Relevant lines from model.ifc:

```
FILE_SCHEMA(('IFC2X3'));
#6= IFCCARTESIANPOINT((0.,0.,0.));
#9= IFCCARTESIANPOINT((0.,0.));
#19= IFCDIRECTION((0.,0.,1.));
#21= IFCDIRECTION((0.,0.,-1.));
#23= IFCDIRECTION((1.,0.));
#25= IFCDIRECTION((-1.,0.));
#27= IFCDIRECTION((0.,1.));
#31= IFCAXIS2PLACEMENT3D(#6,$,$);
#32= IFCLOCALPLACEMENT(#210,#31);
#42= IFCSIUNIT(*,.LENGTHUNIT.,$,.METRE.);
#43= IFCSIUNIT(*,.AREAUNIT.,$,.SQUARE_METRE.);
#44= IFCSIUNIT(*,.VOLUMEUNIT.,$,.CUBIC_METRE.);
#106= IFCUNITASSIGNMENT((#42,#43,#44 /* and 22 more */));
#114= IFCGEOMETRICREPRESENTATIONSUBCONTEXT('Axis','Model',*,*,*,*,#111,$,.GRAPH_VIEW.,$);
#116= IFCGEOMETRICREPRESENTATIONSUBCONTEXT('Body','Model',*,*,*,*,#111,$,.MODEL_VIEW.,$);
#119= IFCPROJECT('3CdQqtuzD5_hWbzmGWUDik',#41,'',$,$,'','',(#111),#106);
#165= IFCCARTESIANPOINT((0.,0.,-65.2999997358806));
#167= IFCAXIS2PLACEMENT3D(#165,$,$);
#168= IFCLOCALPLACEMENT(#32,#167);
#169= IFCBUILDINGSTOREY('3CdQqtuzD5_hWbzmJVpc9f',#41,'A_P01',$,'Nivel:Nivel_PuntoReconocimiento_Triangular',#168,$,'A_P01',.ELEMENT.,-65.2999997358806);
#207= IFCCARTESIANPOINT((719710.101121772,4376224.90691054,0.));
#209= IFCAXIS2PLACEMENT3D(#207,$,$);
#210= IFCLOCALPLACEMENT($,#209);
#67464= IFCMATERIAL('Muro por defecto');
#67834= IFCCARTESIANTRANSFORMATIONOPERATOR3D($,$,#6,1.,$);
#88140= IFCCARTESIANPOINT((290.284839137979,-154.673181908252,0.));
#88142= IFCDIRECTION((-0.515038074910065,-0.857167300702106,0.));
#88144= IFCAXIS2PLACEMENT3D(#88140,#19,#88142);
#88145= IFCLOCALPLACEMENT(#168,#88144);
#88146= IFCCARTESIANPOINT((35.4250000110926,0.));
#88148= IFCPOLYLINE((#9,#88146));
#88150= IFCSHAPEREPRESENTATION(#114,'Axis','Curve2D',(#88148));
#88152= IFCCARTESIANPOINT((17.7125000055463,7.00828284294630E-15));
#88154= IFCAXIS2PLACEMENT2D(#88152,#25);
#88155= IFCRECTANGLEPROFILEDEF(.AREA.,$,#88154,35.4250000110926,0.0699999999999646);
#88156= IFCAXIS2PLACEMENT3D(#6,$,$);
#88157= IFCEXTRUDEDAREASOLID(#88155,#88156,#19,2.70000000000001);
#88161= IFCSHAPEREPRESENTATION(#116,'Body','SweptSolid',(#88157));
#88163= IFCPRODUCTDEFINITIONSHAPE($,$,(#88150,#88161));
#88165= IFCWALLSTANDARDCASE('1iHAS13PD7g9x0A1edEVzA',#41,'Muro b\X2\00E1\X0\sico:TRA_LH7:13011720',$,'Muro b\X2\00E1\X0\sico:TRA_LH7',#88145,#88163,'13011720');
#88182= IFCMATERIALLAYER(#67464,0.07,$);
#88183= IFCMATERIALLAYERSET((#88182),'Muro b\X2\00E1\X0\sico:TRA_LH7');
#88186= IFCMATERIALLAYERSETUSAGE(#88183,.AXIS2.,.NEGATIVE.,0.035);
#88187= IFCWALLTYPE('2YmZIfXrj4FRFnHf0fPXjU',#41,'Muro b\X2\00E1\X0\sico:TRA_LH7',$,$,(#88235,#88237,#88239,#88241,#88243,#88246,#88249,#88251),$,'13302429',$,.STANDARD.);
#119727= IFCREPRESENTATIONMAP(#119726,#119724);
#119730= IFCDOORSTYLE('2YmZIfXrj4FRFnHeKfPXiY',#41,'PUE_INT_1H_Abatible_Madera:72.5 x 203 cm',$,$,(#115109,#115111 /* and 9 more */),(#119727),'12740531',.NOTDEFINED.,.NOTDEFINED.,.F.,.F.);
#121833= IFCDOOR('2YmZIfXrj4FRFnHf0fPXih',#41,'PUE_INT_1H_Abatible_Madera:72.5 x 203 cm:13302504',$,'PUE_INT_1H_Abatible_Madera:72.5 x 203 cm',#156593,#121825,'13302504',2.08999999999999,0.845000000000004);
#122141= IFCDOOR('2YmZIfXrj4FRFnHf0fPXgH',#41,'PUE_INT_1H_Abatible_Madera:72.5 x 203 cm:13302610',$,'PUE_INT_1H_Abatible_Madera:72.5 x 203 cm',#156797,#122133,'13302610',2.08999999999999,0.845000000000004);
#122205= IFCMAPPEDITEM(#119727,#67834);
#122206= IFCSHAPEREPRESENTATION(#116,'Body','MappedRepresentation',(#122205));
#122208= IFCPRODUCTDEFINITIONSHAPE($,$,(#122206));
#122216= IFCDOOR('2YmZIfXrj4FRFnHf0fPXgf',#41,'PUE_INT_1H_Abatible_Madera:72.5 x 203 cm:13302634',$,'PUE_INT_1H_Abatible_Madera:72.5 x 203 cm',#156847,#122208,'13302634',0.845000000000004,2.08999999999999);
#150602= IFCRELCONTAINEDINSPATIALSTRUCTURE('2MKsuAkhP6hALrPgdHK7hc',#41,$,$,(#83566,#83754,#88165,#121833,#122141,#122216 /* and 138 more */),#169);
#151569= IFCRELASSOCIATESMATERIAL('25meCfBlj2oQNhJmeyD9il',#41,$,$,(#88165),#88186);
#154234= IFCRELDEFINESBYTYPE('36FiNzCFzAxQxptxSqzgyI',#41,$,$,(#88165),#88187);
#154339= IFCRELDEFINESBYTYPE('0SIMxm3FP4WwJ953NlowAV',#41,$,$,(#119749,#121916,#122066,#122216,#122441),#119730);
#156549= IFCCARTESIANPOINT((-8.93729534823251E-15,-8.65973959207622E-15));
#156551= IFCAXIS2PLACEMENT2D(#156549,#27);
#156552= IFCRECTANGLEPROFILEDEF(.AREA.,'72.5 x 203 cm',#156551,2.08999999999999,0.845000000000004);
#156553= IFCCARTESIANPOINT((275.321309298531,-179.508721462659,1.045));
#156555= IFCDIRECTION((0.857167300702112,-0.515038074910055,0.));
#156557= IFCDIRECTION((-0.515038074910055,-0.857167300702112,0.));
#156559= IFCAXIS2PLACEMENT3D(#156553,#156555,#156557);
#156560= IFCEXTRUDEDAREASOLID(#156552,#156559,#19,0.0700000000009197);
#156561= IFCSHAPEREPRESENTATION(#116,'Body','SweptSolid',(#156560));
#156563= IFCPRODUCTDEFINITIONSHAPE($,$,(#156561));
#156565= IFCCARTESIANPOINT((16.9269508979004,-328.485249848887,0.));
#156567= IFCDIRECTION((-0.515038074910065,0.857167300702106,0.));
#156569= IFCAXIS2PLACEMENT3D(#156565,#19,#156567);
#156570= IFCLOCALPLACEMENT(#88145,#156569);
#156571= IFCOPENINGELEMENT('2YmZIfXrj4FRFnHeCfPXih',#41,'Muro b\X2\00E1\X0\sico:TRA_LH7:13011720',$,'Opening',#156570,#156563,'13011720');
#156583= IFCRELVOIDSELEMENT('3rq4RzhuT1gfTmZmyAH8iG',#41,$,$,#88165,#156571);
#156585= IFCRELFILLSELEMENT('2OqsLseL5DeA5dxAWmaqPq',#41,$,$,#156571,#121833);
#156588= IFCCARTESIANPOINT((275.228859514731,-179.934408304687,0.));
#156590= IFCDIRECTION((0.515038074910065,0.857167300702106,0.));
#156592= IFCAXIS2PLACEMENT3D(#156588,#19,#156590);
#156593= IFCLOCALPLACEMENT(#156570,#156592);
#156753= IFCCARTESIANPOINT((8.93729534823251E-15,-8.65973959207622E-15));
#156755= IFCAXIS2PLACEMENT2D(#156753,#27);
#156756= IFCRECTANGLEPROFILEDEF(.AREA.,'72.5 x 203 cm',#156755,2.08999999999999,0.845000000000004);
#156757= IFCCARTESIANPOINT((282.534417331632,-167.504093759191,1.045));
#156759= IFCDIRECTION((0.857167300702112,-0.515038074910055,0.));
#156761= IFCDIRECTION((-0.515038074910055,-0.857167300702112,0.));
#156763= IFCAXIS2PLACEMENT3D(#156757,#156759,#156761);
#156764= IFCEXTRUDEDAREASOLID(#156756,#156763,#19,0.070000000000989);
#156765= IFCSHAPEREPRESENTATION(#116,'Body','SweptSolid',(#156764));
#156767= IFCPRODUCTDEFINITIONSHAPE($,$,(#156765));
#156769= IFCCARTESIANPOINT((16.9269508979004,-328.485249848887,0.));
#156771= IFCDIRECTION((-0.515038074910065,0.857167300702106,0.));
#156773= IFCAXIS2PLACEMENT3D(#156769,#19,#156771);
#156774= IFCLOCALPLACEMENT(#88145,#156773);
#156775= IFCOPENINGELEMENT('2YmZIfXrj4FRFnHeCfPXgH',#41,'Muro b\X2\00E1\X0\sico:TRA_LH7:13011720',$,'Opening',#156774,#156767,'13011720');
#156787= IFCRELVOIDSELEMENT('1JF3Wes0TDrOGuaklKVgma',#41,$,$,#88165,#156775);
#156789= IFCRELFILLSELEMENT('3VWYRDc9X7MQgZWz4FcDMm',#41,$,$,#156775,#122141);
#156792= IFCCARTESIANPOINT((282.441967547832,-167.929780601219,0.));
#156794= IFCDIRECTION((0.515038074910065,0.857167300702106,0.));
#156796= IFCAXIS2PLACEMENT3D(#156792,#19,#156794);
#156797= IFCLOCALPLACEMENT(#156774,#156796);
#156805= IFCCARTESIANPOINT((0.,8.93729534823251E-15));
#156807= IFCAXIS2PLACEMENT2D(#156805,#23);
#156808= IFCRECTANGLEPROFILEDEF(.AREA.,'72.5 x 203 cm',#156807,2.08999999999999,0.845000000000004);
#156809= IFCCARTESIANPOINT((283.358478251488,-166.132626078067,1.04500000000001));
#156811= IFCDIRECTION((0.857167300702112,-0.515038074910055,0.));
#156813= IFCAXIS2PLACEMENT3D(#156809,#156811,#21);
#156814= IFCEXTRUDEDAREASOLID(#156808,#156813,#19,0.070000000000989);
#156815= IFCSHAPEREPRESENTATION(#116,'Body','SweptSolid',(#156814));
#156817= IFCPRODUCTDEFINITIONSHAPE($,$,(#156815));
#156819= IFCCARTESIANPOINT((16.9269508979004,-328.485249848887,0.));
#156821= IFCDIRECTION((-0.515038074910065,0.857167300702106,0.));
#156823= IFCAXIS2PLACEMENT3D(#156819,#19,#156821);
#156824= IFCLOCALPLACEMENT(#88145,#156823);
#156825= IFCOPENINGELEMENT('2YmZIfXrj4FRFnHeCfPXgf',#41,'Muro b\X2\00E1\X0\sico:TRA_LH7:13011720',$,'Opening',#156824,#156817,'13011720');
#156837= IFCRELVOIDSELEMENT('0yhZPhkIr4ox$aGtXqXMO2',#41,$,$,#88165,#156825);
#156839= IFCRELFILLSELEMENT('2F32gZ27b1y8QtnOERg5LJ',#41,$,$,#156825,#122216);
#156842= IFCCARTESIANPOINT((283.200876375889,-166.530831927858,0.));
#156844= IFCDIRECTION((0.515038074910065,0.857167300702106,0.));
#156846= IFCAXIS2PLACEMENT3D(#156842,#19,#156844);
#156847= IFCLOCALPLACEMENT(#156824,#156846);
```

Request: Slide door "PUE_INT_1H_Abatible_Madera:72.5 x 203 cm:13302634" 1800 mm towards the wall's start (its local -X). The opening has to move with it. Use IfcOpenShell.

```python
import ifcopenshell
import ifcopenshell.api.geometry
import ifcopenshell.util.placement

model = ifcopenshell.open("model.ifc")

door = model.by_guid("2YmZIfXrj4FRFnHf0fPXgf")
opening = door.FillsVoids[0].RelatingOpeningElement
wall = opening.VoidsElements[0].RelatingBuildingElement

wall_matrix = ifcopenshell.util.placement.get_local_placement(wall.ObjectPlacement)
shift = wall_matrix[:3, 0] * -1.8
before = ifcopenshell.util.placement.get_local_placement(door.ObjectPlacement)[:3, 3].copy()

# The door is placed relative to its opening, so it follows when the opening moves.
matrix = ifcopenshell.util.placement.get_local_placement(opening.ObjectPlacement)
matrix[:3, 3] += shift
ifcopenshell.api.geometry.edit_object_placement(
    model, product=opening, matrix=matrix, is_si=False, should_transform_children=True
)

after = ifcopenshell.util.placement.get_local_placement(door.ObjectPlacement)[:3, 3]
print("door moved by", (after - before).round(3) + 0.0)

model.write("model_v2.ifc")
```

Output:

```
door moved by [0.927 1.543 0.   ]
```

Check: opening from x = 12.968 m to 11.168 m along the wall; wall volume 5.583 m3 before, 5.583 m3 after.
